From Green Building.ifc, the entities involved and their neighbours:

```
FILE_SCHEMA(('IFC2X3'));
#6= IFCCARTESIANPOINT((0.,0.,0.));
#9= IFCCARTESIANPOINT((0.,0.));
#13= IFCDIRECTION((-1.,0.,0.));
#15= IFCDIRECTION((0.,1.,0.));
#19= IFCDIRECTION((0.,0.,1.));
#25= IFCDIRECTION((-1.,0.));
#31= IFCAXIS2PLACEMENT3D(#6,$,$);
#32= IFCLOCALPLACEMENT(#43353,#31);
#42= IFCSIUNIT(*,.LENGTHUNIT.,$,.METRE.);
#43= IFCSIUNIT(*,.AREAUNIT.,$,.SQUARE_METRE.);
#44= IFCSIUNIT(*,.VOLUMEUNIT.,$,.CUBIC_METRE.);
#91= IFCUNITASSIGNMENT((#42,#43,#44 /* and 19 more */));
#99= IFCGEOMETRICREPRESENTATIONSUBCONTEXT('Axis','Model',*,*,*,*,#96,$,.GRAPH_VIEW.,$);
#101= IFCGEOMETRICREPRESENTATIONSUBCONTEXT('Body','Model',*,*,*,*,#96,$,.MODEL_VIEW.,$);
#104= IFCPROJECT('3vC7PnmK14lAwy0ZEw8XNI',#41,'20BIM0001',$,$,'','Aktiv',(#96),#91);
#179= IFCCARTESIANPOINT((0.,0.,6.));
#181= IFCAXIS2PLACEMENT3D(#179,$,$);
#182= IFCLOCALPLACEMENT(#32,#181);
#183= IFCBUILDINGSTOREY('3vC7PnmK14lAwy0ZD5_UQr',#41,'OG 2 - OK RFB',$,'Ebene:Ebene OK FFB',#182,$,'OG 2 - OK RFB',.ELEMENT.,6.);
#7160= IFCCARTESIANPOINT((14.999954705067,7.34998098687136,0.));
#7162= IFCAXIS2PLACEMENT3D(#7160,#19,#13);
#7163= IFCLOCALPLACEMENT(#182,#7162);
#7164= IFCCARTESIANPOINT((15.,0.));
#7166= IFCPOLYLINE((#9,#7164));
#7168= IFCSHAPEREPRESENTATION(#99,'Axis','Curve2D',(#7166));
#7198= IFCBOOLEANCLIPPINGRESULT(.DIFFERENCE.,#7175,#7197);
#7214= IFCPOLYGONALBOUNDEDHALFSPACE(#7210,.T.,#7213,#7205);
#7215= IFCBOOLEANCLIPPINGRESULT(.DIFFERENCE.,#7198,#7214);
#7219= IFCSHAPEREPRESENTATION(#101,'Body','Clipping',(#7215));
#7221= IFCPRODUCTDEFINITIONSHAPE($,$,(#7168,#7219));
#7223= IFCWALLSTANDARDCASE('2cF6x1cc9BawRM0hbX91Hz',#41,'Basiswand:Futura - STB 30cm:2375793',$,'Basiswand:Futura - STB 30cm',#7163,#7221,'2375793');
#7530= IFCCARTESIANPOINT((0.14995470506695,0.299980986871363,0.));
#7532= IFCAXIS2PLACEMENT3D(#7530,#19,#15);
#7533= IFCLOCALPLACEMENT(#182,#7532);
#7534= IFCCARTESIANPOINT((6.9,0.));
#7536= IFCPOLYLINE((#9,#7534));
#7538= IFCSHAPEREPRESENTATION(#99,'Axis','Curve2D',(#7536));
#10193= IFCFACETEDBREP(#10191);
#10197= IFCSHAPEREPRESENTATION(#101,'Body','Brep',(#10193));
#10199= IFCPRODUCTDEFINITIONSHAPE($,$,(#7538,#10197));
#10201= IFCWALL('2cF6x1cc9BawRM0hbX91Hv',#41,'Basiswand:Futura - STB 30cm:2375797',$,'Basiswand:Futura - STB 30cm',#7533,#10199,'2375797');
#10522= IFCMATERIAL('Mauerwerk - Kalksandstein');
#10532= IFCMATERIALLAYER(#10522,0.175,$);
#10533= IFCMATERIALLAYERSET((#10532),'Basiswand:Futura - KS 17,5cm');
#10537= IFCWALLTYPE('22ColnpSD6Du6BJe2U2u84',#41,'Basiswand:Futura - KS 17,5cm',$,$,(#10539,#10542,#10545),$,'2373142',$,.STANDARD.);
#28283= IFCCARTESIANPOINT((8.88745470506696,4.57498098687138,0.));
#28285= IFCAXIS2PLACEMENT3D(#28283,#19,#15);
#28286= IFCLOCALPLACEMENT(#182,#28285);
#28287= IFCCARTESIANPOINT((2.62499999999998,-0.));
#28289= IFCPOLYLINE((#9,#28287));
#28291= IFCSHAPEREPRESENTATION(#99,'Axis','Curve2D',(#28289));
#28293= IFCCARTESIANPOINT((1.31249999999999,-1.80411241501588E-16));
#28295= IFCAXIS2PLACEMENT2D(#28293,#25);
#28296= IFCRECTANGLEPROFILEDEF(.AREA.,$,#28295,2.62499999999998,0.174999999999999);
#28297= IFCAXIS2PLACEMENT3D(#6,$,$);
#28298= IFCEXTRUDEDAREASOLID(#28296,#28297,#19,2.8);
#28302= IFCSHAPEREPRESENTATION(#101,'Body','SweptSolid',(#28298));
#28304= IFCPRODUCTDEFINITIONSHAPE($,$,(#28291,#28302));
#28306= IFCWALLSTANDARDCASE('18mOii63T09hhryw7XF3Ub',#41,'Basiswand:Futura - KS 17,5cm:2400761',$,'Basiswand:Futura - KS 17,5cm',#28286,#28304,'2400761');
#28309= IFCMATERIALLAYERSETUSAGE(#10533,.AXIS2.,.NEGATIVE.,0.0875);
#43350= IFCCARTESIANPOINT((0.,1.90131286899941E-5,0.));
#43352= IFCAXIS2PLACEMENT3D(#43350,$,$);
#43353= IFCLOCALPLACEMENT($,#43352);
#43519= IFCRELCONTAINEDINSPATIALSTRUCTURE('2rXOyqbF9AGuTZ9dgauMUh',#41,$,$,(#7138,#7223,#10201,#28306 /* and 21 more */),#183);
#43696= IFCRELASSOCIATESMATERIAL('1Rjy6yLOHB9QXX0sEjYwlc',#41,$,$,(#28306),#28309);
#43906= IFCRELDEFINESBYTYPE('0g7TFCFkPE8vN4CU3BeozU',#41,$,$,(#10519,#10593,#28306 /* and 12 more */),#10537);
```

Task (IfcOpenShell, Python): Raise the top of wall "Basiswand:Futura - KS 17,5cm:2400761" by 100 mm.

```python
import ifcopenshell
import ifcopenshell.geom
import ifcopenshell.util.representation
import ifcopenshell.util.shape

model = ifcopenshell.open("Green Building.ifc")
settings = ifcopenshell.geom.settings()


def volume(element):
    """Net volume in cubic metres, openings subtracted."""
    shape = ifcopenshell.geom.create_shape(settings, element)
    return ifcopenshell.util.shape.get_volume(shape.geometry)


wall = model.by_guid("18mOii63T09hhryw7XF3Ub")
before = volume(wall)

body = ifcopenshell.util.representation.get_representation(wall, "Model", "Body")
solid = body.Items[0]
old_height = solid.Depth
solid.Depth += 0.1
after = volume(wall)

print(f"height {old_height:g} -> {solid.Depth:g}, volume {before:.3f} -> {after:.3f} m3")

model.write("Green Building_rev.ifc")
```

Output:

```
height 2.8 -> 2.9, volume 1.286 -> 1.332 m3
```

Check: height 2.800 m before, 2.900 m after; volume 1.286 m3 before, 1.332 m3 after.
